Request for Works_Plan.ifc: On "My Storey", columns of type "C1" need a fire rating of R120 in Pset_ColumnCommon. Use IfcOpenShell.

First a look at what the model holds.

```python
import ifcopenshell
import ifcopenshell.util.element

model = ifcopenshell.open("Works_Plan.ifc")
print(model.schema)
storey = next(s for s in model.by_type("IfcBuildingStorey") if s.Name == "My Storey")
columns = [e for e in ifcopenshell.util.element.get_decomposition(storey) if e.is_a("IfcColumn")]
seen = {}
for e in columns:
    element_type = ifcopenshell.util.element.get_type(e)
    key = (element_type.Name if element_type != e and element_type else None, ifcopenshell.util.element.get_pset(e, "Pset_ColumnCommon", "FireRating"))
    seen[key] = seen.get(key, 0) + 1
for (name, value), count in sorted(seen.items(), key=str):
    print(count, "x", name, "|", value)
```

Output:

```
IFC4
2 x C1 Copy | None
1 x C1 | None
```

```python
import ifcopenshell
import ifcopenshell.api.pset
import ifcopenshell.util.element

model = ifcopenshell.open("Works_Plan.ifc")

storey = next(s for s in model.by_type("IfcBuildingStorey") if s.Name == "My Storey")
columns = [e for e in ifcopenshell.util.element.get_decomposition(storey) if e.is_a("IfcColumn")]

count = 0
for e in columns:
    element_type = ifcopenshell.util.element.get_type(e)
    if element_type in (None, e) or element_type.Name != "C1":
        continue
    # add_pset returns the element's existing set when there is one.
    pset = ifcopenshell.api.pset.add_pset(model, product=e, name="Pset_ColumnCommon")
    ifcopenshell.api.pset.edit_pset(model, pset=pset, properties={"FireRating": "R120"})
    count += 1

print(count, "columns updated")

model.write("Works_Plan_v2.ifc")
```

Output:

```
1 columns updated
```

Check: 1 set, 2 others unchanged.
